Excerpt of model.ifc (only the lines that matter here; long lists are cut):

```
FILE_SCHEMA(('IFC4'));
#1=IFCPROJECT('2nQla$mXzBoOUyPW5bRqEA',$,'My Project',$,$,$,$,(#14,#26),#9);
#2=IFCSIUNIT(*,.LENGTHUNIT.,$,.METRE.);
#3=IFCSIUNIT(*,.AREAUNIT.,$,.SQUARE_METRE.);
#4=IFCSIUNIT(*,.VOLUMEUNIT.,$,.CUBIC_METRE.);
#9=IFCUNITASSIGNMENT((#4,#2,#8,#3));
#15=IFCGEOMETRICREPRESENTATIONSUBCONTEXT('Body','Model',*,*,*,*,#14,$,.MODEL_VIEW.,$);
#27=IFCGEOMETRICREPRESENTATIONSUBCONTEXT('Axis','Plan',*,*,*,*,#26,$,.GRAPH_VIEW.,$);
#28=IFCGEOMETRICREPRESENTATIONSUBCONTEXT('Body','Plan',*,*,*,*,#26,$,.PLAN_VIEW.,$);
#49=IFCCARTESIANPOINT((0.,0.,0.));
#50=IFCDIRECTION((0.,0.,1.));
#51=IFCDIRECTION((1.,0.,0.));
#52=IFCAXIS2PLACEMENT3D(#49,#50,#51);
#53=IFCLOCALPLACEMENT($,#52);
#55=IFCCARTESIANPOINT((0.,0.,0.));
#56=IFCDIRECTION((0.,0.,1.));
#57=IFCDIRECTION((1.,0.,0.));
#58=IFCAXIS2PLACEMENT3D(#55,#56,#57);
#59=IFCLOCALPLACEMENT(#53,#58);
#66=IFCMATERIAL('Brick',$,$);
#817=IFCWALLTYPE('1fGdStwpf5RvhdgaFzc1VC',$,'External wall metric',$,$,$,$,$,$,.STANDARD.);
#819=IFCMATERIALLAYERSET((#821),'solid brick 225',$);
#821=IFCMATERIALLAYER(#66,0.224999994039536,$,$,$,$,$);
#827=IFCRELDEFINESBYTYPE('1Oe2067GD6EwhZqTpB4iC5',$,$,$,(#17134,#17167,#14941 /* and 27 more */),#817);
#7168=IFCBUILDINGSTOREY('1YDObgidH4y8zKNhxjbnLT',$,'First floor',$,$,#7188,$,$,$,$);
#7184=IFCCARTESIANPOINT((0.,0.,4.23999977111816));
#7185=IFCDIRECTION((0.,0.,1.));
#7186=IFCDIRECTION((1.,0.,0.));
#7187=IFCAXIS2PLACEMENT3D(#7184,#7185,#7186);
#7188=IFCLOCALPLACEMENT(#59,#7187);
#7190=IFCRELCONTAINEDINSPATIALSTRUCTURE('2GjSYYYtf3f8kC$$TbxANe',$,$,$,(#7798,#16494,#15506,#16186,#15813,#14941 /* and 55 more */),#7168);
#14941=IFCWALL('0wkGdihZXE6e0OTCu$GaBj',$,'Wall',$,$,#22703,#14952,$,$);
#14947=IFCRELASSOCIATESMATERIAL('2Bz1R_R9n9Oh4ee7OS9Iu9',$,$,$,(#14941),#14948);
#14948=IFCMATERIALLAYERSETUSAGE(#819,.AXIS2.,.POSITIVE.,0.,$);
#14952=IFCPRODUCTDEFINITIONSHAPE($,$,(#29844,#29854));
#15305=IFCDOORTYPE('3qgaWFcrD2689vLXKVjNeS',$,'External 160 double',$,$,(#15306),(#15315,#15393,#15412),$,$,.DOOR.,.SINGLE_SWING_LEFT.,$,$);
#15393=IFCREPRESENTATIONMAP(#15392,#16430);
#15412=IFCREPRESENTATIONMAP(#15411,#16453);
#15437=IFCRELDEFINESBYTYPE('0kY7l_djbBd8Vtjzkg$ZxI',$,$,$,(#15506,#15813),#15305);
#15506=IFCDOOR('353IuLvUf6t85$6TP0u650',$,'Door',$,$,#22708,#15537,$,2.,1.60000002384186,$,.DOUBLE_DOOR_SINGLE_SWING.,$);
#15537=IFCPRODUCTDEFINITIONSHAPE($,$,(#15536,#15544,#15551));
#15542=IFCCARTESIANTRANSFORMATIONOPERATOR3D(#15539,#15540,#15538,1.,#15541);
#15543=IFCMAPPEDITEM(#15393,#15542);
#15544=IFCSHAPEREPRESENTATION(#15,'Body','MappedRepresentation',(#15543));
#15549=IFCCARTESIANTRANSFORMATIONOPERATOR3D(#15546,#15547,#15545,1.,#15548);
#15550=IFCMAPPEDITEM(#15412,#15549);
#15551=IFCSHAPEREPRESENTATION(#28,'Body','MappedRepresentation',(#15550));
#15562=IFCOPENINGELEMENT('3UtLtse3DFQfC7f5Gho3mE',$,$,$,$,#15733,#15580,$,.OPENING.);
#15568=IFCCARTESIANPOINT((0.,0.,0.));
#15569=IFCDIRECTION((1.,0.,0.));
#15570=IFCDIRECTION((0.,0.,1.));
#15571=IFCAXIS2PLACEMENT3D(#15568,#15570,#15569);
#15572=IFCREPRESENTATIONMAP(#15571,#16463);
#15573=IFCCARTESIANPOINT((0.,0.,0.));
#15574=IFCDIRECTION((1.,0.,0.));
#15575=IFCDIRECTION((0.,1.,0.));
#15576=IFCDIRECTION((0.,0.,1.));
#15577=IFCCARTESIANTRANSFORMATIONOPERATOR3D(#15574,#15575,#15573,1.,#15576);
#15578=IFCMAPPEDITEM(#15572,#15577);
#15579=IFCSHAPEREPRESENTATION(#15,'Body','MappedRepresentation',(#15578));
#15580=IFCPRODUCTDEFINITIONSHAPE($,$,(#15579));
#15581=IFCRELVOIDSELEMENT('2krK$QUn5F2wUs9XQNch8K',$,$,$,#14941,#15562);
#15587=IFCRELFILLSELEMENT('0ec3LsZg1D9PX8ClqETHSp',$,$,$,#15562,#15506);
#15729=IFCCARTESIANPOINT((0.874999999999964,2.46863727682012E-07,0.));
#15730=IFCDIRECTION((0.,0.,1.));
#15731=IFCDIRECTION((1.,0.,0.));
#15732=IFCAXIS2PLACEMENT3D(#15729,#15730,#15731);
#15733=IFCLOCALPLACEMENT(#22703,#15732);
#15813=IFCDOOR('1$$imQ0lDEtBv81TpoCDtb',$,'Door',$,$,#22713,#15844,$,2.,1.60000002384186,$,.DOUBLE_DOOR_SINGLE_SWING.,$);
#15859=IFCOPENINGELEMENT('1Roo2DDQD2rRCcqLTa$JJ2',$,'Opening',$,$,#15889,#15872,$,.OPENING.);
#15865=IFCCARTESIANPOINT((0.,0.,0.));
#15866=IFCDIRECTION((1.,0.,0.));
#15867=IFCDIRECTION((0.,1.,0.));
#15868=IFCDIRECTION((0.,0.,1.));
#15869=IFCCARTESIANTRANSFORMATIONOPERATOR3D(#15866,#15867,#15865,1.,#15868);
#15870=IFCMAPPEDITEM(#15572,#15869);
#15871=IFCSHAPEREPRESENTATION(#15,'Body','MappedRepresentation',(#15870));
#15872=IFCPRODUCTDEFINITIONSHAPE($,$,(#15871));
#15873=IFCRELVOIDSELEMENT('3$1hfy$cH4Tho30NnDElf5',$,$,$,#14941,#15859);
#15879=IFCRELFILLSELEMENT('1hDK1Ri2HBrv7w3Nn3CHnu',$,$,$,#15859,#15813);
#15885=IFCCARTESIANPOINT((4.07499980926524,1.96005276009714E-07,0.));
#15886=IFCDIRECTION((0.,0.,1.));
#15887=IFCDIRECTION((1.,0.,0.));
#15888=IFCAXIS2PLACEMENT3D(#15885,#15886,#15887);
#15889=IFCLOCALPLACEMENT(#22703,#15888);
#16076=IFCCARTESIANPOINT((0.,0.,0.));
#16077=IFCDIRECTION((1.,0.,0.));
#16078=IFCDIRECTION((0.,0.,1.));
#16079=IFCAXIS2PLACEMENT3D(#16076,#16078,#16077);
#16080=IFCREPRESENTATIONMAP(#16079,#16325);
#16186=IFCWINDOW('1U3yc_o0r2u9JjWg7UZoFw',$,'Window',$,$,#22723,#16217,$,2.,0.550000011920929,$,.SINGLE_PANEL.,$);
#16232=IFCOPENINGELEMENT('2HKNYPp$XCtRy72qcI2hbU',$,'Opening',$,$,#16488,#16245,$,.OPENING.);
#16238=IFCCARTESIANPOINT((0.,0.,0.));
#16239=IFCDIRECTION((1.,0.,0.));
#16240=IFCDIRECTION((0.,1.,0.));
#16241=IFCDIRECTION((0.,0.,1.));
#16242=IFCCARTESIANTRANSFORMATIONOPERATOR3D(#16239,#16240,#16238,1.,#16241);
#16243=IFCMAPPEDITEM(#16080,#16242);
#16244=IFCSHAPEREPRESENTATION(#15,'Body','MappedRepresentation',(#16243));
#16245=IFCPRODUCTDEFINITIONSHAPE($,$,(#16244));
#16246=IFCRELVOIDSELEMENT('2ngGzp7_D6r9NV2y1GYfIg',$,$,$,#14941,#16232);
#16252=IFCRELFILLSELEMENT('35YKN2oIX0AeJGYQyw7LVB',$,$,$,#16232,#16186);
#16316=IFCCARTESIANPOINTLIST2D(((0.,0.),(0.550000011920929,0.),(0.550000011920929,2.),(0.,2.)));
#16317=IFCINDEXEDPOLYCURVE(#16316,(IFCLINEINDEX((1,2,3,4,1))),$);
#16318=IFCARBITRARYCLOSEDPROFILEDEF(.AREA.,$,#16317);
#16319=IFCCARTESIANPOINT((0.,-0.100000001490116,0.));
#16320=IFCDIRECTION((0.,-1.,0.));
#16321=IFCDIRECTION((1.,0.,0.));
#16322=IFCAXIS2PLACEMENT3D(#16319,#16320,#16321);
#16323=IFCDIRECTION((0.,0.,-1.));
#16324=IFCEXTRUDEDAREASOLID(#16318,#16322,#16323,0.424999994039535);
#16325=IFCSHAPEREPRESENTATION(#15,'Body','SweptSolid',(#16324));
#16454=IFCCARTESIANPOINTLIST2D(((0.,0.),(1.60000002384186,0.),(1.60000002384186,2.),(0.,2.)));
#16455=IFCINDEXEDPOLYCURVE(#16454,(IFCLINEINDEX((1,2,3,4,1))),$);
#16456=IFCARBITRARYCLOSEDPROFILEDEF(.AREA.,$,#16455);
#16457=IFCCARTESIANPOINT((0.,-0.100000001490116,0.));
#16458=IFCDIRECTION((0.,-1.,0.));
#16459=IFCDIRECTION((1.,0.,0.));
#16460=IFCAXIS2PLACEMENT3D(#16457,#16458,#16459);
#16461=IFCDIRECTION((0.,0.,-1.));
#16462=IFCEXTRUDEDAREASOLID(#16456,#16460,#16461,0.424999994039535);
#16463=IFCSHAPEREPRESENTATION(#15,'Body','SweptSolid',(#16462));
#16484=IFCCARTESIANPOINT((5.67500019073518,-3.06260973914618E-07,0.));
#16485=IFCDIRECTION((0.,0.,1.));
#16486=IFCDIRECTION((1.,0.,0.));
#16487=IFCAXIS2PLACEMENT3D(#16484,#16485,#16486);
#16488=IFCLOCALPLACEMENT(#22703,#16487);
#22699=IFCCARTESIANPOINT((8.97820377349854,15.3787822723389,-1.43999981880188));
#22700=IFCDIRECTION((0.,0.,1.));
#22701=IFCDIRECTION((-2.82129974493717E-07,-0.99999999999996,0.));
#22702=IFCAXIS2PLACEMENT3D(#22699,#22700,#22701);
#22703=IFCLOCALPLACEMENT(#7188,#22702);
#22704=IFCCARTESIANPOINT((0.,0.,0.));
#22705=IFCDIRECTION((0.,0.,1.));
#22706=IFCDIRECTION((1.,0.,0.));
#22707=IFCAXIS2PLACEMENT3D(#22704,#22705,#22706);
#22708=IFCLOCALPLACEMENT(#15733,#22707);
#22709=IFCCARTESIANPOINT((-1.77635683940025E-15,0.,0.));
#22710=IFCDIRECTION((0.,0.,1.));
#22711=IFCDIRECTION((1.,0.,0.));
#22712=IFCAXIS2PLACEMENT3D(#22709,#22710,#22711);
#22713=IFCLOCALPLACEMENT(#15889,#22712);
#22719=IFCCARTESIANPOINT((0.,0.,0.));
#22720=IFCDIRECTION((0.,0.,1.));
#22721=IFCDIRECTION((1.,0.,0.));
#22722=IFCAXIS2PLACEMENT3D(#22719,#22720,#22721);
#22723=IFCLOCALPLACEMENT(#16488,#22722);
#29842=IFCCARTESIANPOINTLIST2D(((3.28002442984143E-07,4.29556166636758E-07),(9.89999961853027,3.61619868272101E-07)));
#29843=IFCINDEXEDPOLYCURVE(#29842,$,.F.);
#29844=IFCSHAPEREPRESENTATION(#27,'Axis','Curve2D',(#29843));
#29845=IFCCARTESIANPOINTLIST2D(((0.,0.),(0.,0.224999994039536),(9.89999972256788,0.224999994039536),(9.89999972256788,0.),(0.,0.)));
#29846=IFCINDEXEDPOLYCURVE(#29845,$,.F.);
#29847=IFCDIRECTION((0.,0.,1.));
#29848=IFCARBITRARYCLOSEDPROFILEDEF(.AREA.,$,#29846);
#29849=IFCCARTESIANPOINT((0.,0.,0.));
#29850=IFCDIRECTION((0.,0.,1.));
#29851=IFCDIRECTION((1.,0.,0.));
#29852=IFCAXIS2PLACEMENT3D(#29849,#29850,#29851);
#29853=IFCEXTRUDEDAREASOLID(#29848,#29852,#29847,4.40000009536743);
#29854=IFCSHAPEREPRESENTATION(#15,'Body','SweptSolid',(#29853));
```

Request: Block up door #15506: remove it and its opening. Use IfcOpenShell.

```python
import ifcopenshell
import ifcopenshell.api.feature
import ifcopenshell.api.root
import ifcopenshell.geom
import ifcopenshell.util.shape

model = ifcopenshell.open("model.ifc")
settings = ifcopenshell.geom.settings()


def volume(element):
    """Net volume in cubic metres, openings subtracted."""
    shape = ifcopenshell.geom.create_shape(settings, element)
    return ifcopenshell.util.shape.get_volume(shape.geometry)


door = model.by_guid("353IuLvUf6t85$6TP0u650")
opening = door.FillsVoids[0].RelatingOpeningElement
wall = opening.VoidsElements[0].RelatingBuildingElement
before = volume(wall)

ifcopenshell.api.root.remove_product(model, product=door)
ifcopenshell.api.feature.remove_feature(model, feature=opening)

after = volume(wall)

print(f"wall volume {before:.3f} -> {after:.3f} m3")

model.write("model_updated.ifc")
```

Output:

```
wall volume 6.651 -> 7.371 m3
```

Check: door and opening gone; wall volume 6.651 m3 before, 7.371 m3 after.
